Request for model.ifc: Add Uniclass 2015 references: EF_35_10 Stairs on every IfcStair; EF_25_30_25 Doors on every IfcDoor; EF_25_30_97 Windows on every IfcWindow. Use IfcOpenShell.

First a look at what the model holds.

```python
import ifcopenshell

model = ifcopenshell.open("model.ifc")
print(model.schema)
print("classifications:", [c.Name for c in model.by_type("IfcClassification")])
for ifc_class in ("IfcDoor", "IfcRoof", "IfcStair", "IfcWall", "IfcWindow"):
    print(ifc_class, len(model.by_type(ifc_class)))
```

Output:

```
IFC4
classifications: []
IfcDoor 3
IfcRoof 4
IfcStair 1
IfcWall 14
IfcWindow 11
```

```python
import ifcopenshell
import ifcopenshell.api.classification

model = ifcopenshell.open("model.ifc")

system = ifcopenshell.api.classification.add_classification(model, classification="Uniclass 2015")

codes = {
    "IfcStair": ("EF_35_10", "Stairs"),
    "IfcDoor": ("EF_25_30_25", "Doors"),
    "IfcWindow": ("EF_25_30_97", "Windows"),
}
for ifc_class, (code, name) in codes.items():
    products = model.by_type(ifc_class)
    ifcopenshell.api.classification.add_reference(
        model, products=products, classification=system, identification=code, name=name
    )
    print(code, len(products))

model.write("model-out.ifc")
```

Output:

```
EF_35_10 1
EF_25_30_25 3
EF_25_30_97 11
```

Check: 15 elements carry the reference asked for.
